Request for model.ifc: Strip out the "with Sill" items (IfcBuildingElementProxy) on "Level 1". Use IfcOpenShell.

First a look at what the model holds.

```python
import ifcopenshell
import ifcopenshell.util.element

model = ifcopenshell.open("model.ifc")
print(model.schema)
storey = next(s for s in model.by_type("IfcBuildingStorey") if s.Name == "Level 1")
proxies = [e for e in ifcopenshell.util.element.get_decomposition(storey) if e.is_a("IfcBuildingElementProxy")]
seen = {}
for e in proxies:
    element_type = ifcopenshell.util.element.get_type(e)
    name = element_type.Name if element_type not in (None, e) else None
    seen[name] = seen.get(name, 0) + 1
for name, count in sorted(seen.items(), key=str):
    print(count, "x", name)
```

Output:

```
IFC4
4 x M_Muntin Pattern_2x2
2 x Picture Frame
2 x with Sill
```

```python
import ifcopenshell
import ifcopenshell.api.root
import ifcopenshell.util.element

model = ifcopenshell.open("model.ifc")

storey = next(s for s in model.by_type("IfcBuildingStorey") if s.Name == "Level 1")
proxies = [e for e in ifcopenshell.util.element.get_decomposition(storey) if e.is_a("IfcBuildingElementProxy")]
targets = [e for e in proxies if (t := ifcopenshell.util.element.get_type(e)) not in (None, e) and t.Name == "with Sill"]

for e in targets:
    ifcopenshell.api.root.remove_product(model, product=e)
print(len(targets), "removed")

model.write("model_rev.ifc")
```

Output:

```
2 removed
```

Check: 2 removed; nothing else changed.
